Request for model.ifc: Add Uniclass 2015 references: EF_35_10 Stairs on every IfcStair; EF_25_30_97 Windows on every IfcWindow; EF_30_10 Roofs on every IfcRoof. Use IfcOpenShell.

First a look at what the model holds.

```python
import ifcopenshell

model = ifcopenshell.open("model.ifc")
print(model.schema)
print("classifications:", [c.Name for c in model.by_type("IfcClassification")])
for ifc_class in ("IfcDoor", "IfcRoof", "IfcStair", "IfcWall", "IfcWindow"):
    print(ifc_class, len(model.by_type(ifc_class)))
```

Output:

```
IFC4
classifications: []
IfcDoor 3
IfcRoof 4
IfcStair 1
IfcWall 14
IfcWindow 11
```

```python
import ifcopenshell
import ifcopenshell.api.classification

model = ifcopenshell.open("model.ifc")

system = ifcopenshell.api.classification.add_classification(model, classification="Uniclass 2015")

codes = {
    "IfcStair": ("EF_35_10", "Stairs"),
    "IfcWindow": ("EF_25_30_97", "Windows"),
    "IfcRoof": ("EF_30_10", "Roofs"),
}
for ifc_class, (code, name) in codes.items():
    products = model.by_type(ifc_class)
    ifcopenshell.api.classification.add_reference(
        model, products=products, classification=system, identification=code, name=name
    )
    print(code, len(products))

model.write("model_edited.ifc")
```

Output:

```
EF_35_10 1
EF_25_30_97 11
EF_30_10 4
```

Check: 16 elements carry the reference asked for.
